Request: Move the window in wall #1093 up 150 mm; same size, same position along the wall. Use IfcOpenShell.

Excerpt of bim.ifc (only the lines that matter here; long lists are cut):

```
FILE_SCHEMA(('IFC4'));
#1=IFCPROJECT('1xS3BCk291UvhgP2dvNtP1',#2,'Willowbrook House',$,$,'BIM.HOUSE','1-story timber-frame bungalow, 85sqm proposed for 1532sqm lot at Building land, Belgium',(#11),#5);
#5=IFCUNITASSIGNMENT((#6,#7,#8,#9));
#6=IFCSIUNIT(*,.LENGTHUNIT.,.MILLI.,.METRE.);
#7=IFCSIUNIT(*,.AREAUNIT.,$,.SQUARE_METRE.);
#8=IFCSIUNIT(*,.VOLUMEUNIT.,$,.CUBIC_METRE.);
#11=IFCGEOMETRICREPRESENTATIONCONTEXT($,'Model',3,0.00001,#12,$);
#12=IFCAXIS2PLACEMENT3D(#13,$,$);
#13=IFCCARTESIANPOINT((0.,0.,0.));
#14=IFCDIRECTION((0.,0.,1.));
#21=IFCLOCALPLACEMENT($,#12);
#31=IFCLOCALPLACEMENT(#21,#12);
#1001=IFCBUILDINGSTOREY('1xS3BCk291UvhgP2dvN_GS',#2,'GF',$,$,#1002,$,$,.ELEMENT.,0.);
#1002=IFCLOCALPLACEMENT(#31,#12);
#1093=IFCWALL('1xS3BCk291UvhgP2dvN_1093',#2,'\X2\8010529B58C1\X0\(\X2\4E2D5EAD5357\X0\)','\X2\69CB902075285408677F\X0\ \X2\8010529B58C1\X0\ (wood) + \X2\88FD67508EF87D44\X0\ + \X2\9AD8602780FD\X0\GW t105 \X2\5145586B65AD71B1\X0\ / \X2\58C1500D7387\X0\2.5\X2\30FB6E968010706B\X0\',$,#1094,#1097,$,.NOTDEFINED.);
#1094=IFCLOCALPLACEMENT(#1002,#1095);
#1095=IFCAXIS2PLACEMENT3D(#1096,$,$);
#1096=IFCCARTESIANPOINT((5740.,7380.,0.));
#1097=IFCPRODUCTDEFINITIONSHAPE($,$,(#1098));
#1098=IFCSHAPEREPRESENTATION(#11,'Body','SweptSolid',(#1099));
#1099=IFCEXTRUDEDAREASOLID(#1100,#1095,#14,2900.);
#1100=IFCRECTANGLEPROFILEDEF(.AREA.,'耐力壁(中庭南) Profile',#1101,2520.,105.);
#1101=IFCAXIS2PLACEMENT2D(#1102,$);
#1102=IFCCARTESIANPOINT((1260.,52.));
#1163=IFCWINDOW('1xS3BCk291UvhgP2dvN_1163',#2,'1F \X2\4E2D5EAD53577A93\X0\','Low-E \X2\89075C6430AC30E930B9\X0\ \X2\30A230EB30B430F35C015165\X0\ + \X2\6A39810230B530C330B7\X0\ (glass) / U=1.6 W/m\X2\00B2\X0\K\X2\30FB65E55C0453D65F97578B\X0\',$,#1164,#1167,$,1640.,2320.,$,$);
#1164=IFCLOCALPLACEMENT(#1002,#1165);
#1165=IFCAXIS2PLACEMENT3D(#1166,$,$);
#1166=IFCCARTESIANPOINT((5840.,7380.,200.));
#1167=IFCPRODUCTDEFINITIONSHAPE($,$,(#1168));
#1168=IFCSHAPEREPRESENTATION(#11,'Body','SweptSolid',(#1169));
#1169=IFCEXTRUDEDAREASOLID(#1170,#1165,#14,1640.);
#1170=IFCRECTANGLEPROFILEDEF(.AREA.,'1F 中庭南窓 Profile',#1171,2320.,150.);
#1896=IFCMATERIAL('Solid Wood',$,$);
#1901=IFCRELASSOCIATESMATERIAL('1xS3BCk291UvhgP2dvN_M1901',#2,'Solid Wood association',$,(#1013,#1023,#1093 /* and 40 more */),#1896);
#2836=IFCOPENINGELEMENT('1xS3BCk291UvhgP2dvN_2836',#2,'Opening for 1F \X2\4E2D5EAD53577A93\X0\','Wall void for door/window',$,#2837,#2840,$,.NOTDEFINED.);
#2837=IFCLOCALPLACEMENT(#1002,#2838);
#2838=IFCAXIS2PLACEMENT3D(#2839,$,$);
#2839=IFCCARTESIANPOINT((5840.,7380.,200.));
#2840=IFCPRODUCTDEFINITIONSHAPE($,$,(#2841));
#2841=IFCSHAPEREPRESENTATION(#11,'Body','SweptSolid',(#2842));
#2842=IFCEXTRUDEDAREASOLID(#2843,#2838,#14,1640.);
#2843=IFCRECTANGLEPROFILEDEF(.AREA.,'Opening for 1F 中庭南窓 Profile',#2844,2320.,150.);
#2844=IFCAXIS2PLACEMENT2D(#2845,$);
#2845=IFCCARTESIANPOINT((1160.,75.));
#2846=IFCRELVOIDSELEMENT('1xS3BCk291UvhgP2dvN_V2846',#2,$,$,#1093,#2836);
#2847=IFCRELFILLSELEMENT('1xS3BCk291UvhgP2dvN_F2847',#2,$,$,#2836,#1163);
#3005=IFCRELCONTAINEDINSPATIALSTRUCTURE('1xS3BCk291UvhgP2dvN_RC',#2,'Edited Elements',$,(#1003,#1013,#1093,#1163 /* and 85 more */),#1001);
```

```python
import numpy as np
import ifcopenshell
import ifcopenshell.api.geometry
import ifcopenshell.util.placement
import ifcopenshell.util.unit

model = ifcopenshell.open("bim.ifc")
unit_scale = ifcopenshell.util.unit.calculate_unit_scale(model)

window = model.by_id(1163)
opening = window.FillsVoids[0].RelatingOpeningElement
dz = 0.15 / unit_scale

shift = np.array([0.0, 0.0, dz])
# The window is not placed relative to its opening, so move both.
for product in (opening, window):
    matrix = ifcopenshell.util.placement.get_local_placement(product.ObjectPlacement)
    matrix[:3, 3] += shift
    ifcopenshell.api.geometry.edit_object_placement(model, product=product, matrix=matrix, is_si=False)

print(f"moved by {dz * unit_scale:+.3f} m")

model.write("bim_edited.ifc")
```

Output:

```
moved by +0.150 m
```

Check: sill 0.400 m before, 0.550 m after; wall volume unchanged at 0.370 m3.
